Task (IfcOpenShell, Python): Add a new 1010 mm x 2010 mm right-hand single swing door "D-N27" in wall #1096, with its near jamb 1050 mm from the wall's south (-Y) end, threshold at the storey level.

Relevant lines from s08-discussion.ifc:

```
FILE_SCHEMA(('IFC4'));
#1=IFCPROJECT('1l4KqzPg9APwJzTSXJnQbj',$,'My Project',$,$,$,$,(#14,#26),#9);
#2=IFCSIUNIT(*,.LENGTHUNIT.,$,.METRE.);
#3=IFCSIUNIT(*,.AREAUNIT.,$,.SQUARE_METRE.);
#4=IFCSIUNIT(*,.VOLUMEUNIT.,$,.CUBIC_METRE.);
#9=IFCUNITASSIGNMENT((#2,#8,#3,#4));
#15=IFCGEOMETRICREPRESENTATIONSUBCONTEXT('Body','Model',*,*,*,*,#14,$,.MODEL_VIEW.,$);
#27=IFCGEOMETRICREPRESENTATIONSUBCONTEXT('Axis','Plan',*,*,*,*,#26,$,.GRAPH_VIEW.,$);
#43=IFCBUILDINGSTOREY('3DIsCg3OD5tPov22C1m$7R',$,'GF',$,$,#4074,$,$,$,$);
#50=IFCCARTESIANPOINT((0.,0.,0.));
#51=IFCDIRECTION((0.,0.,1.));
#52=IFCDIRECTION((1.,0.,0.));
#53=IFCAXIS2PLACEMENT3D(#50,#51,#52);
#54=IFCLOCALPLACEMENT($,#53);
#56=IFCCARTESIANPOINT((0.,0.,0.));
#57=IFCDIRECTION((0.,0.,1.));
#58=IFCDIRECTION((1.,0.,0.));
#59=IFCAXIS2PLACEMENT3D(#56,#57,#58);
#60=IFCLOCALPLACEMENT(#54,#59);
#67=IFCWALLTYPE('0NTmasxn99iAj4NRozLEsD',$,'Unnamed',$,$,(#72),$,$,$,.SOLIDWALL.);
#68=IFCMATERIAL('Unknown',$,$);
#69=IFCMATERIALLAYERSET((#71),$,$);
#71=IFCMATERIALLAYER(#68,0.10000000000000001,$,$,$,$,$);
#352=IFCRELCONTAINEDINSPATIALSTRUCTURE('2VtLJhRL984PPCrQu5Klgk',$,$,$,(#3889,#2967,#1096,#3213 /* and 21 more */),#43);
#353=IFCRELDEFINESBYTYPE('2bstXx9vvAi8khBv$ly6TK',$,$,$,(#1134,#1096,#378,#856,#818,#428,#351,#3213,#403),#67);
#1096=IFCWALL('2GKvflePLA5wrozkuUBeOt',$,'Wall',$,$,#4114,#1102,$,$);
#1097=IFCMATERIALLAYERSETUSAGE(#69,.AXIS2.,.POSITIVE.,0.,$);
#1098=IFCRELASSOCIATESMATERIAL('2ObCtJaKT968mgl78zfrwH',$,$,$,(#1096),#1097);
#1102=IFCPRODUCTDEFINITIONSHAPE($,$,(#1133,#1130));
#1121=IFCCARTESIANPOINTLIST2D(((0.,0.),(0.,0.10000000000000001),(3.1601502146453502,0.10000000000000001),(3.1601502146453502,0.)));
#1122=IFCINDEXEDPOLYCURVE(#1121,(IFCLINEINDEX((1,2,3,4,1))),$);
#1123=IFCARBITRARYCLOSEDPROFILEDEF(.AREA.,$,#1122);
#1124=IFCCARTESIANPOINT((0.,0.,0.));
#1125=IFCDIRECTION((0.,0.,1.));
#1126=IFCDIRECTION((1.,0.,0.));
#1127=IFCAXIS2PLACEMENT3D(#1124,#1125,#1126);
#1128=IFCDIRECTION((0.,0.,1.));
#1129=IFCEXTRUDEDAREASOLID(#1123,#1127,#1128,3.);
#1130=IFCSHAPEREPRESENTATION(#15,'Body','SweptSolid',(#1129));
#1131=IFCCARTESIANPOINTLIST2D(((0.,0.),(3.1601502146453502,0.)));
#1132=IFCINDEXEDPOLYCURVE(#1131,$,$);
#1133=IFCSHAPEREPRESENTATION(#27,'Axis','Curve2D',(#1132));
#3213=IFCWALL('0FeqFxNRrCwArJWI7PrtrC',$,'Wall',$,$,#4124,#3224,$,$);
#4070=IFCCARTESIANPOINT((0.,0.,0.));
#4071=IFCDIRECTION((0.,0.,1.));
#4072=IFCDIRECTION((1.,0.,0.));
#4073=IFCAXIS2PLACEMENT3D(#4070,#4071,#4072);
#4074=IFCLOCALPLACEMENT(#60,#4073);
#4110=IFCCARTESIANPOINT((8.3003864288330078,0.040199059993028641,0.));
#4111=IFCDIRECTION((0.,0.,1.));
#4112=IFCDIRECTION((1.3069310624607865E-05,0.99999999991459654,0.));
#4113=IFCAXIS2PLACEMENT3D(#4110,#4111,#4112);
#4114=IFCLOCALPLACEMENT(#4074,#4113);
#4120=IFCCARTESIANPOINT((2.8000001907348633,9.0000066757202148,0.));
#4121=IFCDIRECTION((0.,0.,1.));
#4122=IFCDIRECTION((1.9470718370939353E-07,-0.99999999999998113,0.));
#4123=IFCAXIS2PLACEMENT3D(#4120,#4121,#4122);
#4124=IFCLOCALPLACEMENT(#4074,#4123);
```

```python
import numpy as np
import ifcopenshell
import ifcopenshell.api.feature
import ifcopenshell.api.geometry
import ifcopenshell.api.root
import ifcopenshell.api.spatial
import ifcopenshell.geom
import ifcopenshell.util.element
import ifcopenshell.util.placement
import ifcopenshell.util.representation
import ifcopenshell.util.shape
import ifcopenshell.util.unit

model = ifcopenshell.open("s08-discussion.ifc")
unit_scale = ifcopenshell.util.unit.calculate_unit_scale(model)
settings = ifcopenshell.geom.settings()


def volume(element):
    """Net volume in cubic metres, openings subtracted."""
    shape = ifcopenshell.geom.create_shape(settings, element)
    return ifcopenshell.util.shape.get_volume(shape.geometry)


wall = model.by_guid("2GKvflePLA5wrozkuUBeOt")
storey = ifcopenshell.util.element.get_container(wall, ifc_class="IfcBuildingStorey")
context = ifcopenshell.util.representation.get_context(model, "Model", "Body", "MODEL_VIEW")
before = volume(wall)

width, height, from_end, sill = 1.01, 2.01, 1.05, 0.0  # metres

# The wall runs along its own X axis, and the end named is its -X end.
wall_shape = ifcopenshell.geom.create_shape(settings, wall)
x, y, z = ifcopenshell.util.shape.get_vertices(wall_shape.geometry).T
start = x.min() + from_end
face, thickness = float(y.min()), float(y.max() - y.min())
wall_matrix = ifcopenshell.util.placement.get_local_placement(wall.ObjectPlacement)
level = ifcopenshell.util.placement.get_local_placement(storey.ObjectPlacement)[2, 3]


def in_wall(x, y):
    """Placement at x, y metres in the wall's axes, at sill height."""
    matrix = wall_matrix.copy()
    matrix[:, 3] = wall_matrix @ np.array([x / unit_scale, y / unit_scale, 0.0, 1.0])
    matrix[2, 3] = level + sill / unit_scale
    return matrix


# Opening: a box that overshoots both wall faces by 50 mm.
opening = ifcopenshell.api.root.create_entity(model, ifc_class="IfcOpeningElement", predefined_type="OPENING")
box = ifcopenshell.api.geometry.add_wall_representation(
    model, context=context, length=width, height=height, thickness=thickness + 0.1
)
ifcopenshell.api.geometry.assign_representation(model, product=opening, representation=box)
ifcopenshell.api.geometry.edit_object_placement(model, product=opening, matrix=in_wall(start, face - 0.05), is_si=False)
ifcopenshell.api.feature.add_feature(model, feature=opening, element=wall)

door = ifcopenshell.api.root.create_entity(model, ifc_class="IfcDoor", name="D-N27", predefined_type="DOOR")
door.OverallWidth, door.OverallHeight = width / unit_scale, height / unit_scale
door.OperationType = "SINGLE_SWING_RIGHT"
body = ifcopenshell.api.geometry.add_door_representation(
    model,
    context=context,
    overall_width=door.OverallWidth,
    overall_height=door.OverallHeight,
    operation_type="SINGLE_SWING_RIGHT",
    lining_properties={"LiningDepth": thickness / unit_scale, "ThresholdDepth": thickness / unit_scale},
)
ifcopenshell.api.geometry.assign_representation(model, product=door, representation=body)
ifcopenshell.api.spatial.assign_container(model, products=[door], relating_structure=storey)
ifcopenshell.api.feature.add_filling(model, opening=opening, element=door)

# The lining spans the wall, so the door starts at the wall face.
ifcopenshell.api.geometry.edit_object_placement(model, product=door, matrix=in_wall(start, face), is_si=False)

after = volume(wall)

print(f"wall volume {before:.3f} -> {after:.3f} m3")

model.write("s08-discussion-out.ifc")
```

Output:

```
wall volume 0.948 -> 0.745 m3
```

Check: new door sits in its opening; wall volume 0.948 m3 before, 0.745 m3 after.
